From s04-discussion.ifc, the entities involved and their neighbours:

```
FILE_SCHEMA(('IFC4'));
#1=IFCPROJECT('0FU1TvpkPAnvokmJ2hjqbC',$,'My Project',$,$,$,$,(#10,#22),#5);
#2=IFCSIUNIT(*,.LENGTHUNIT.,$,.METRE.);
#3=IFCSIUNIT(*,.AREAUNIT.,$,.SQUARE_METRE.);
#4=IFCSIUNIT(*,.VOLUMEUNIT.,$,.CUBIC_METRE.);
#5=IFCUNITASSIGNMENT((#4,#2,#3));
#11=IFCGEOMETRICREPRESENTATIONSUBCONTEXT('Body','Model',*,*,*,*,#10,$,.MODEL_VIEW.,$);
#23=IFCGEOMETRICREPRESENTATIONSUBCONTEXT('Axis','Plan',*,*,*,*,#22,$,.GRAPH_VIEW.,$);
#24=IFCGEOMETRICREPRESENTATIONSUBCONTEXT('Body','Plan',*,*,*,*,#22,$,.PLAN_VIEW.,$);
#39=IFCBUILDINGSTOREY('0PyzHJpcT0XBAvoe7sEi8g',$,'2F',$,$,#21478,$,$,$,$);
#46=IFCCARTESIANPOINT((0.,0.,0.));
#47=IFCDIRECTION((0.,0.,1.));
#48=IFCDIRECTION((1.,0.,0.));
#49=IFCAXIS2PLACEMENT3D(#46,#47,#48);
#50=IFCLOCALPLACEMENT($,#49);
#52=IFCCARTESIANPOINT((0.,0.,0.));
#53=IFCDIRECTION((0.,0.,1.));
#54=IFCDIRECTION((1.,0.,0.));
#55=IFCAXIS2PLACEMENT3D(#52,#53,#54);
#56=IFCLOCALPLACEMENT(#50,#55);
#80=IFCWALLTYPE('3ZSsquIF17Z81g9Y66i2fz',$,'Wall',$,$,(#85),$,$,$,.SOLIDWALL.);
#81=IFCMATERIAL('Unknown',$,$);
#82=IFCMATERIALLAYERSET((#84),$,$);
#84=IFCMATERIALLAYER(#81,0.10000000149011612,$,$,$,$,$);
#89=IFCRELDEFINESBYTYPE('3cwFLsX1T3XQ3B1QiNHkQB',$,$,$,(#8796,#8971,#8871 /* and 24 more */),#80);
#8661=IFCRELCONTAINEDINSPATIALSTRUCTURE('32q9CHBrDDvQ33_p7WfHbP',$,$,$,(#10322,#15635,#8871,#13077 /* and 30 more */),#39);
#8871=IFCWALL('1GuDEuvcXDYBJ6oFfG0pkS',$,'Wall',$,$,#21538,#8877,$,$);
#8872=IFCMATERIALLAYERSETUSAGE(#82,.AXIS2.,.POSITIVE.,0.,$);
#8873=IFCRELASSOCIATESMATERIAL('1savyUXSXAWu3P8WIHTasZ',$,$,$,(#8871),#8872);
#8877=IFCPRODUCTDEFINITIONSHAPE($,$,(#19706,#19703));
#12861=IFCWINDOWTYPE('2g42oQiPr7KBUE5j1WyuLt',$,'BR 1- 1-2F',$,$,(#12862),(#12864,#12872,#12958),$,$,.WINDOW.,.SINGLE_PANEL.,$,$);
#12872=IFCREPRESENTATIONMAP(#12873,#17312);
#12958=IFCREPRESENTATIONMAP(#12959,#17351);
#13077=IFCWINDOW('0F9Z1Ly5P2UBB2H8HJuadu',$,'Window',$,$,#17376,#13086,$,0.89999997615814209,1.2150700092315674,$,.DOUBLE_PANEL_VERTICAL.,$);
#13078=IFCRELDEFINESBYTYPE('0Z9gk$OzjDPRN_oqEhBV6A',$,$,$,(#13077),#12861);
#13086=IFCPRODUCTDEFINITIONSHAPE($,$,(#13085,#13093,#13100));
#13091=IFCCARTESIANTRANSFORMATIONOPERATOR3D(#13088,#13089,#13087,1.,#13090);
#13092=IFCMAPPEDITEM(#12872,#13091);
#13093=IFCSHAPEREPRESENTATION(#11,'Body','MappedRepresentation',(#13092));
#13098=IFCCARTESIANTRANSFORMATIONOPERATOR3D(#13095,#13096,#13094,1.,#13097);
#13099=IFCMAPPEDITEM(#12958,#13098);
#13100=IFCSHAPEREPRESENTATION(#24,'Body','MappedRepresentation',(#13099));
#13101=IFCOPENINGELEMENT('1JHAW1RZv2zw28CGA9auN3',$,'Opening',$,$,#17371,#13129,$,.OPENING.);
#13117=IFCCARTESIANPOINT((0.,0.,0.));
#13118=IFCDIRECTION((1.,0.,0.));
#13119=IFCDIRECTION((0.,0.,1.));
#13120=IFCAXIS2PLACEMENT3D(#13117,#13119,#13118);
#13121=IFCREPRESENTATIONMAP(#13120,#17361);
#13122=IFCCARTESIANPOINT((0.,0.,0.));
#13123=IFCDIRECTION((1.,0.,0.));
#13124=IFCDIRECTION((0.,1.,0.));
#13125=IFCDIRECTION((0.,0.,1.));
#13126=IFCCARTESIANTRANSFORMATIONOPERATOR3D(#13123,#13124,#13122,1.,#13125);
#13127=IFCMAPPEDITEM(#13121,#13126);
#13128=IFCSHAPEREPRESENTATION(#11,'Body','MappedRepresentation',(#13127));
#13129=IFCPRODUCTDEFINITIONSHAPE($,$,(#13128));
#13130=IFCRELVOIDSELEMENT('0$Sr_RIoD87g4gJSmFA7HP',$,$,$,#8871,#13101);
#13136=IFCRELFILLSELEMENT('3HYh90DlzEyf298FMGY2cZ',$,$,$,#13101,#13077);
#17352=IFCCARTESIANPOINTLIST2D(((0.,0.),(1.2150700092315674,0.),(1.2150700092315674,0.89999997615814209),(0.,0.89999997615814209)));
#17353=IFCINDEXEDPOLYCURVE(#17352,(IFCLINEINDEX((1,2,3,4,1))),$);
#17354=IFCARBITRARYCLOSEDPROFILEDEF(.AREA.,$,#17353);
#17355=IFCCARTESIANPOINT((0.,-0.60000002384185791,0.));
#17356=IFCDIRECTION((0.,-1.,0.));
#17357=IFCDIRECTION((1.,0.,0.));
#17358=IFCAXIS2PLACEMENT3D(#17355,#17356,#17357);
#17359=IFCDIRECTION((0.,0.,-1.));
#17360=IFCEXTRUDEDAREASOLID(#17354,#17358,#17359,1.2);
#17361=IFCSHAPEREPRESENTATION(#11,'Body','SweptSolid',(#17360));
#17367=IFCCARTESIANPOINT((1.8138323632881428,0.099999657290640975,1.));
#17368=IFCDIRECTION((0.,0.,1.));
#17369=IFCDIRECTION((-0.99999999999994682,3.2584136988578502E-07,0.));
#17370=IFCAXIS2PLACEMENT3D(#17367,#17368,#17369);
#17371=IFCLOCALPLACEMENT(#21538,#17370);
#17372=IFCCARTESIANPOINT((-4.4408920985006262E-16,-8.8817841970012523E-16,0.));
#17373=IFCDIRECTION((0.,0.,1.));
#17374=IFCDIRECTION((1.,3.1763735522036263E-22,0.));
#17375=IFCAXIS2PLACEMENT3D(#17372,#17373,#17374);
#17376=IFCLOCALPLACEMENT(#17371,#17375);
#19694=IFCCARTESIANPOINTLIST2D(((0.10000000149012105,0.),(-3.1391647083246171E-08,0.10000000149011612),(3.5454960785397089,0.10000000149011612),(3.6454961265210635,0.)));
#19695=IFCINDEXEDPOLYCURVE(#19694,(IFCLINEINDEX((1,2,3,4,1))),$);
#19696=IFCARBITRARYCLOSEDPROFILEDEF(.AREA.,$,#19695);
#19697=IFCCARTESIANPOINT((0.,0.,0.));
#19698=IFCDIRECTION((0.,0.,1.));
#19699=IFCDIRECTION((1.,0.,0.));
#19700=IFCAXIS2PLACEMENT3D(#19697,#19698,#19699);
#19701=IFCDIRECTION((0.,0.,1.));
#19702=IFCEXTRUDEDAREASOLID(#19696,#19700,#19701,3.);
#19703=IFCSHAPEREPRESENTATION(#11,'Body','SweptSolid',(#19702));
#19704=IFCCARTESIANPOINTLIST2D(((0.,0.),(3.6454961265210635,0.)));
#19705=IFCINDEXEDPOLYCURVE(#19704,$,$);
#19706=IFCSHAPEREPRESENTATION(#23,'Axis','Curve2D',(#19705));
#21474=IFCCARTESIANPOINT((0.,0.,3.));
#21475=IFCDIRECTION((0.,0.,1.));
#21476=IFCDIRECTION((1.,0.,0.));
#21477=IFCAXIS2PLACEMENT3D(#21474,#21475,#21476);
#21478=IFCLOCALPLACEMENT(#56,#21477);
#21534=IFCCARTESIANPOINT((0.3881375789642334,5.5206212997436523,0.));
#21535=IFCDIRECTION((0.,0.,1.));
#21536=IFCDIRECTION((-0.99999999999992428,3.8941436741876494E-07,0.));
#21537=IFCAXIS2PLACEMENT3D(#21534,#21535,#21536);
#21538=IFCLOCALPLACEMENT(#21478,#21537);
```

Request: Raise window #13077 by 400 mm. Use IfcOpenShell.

```python
import numpy as np
import ifcopenshell
import ifcopenshell.api.geometry
import ifcopenshell.util.placement
import ifcopenshell.util.unit

model = ifcopenshell.open("s04-discussion.ifc")
unit_scale = ifcopenshell.util.unit.calculate_unit_scale(model)

window = model.by_id(13077)
opening = window.FillsVoids[0].RelatingOpeningElement
dz = 0.4 / unit_scale

shift = np.array([0.0, 0.0, dz])
# The window is placed relative to its opening, so it follows when the opening moves.
matrix = ifcopenshell.util.placement.get_local_placement(opening.ObjectPlacement)
matrix[:3, 3] += shift
ifcopenshell.api.geometry.edit_object_placement(
    model, product=opening, matrix=matrix, is_si=False, should_transform_children=True
)

print(f"moved by {dz * unit_scale:+.3f} m")

model.write("s04-discussion_updated.ifc")
```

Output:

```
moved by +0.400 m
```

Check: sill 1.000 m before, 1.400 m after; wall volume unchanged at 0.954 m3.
